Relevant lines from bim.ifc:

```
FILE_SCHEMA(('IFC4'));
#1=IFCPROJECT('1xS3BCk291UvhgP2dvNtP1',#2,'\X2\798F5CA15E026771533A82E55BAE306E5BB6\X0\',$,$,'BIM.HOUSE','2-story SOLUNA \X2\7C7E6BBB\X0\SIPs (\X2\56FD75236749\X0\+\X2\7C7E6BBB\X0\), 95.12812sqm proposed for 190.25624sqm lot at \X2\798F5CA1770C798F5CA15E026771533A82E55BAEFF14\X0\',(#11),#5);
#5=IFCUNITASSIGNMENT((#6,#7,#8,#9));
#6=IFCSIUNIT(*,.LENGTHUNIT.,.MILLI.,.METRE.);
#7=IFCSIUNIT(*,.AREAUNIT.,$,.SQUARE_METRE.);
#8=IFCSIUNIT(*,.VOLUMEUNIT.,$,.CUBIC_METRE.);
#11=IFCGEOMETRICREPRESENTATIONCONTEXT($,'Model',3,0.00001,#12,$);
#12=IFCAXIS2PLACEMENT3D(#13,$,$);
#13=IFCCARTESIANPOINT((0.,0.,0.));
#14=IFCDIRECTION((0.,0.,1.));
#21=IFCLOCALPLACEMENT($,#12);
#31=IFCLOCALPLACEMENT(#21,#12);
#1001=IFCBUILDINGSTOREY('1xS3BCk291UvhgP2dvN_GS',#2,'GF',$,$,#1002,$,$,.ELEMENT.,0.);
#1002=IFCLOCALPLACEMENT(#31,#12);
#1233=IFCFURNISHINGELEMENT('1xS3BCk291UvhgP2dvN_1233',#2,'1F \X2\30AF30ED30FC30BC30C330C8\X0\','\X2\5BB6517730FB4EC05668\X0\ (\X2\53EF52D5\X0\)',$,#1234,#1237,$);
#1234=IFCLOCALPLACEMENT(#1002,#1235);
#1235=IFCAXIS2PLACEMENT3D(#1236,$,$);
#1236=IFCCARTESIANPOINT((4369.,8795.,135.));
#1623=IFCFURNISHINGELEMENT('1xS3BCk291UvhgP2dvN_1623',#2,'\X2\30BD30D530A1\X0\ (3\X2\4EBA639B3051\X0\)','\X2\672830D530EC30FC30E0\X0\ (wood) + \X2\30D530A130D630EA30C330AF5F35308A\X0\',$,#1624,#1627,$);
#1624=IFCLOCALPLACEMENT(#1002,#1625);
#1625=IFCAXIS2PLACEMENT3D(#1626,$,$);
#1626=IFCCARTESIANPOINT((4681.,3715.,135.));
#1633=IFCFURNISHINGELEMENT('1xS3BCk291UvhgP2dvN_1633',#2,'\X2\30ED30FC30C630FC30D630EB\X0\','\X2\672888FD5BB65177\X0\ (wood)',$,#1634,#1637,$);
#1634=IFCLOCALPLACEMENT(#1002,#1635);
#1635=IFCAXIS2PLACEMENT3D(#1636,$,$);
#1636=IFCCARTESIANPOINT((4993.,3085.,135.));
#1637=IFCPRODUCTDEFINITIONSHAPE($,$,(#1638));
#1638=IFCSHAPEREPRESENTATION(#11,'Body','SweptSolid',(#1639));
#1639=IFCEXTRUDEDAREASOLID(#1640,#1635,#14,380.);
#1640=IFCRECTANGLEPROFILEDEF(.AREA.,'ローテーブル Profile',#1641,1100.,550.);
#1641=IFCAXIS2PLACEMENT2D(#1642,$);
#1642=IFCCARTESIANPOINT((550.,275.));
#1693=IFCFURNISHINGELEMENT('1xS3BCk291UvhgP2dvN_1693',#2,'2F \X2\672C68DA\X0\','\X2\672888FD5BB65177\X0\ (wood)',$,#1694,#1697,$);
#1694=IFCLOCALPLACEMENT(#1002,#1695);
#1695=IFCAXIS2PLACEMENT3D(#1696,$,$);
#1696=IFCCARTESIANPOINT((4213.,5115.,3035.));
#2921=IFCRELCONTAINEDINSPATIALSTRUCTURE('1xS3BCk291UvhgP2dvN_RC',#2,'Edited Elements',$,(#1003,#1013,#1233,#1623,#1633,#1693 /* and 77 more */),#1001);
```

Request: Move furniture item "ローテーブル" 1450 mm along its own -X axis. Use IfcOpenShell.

```python
import ifcopenshell
import ifcopenshell.api.geometry
import ifcopenshell.util.placement

model = ifcopenshell.open("bim.ifc")

item = model.by_id(1633)
matrix = ifcopenshell.util.placement.get_local_placement(item.ObjectPlacement)
matrix[:3, 3] -= matrix[:3, 0] * 1450.0
ifcopenshell.api.geometry.edit_object_placement(model, product=item, matrix=matrix, is_si=False)

print(ifcopenshell.util.placement.get_local_placement(item.ObjectPlacement).round(3) + 0.0)

model.write("bim-out.ifc")
```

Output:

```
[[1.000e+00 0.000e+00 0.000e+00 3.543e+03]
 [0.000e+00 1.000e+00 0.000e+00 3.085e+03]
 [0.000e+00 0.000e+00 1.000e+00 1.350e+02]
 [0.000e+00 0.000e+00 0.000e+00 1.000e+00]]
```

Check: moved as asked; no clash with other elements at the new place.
